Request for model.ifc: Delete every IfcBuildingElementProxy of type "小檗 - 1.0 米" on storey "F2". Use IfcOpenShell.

First a look at what the model holds.

```python
import ifcopenshell
import ifcopenshell.util.element

model = ifcopenshell.open("model.ifc")
print(model.schema)
storey = next(s for s in model.by_type("IfcBuildingStorey") if s.Name == "F2")
proxies = [e for e in ifcopenshell.util.element.get_decomposition(storey) if e.is_a("IfcBuildingElementProxy")]
seen = {}
for e in proxies:
    element_type = ifcopenshell.util.element.get_type(e)
    name = element_type.Name if element_type not in (None, e) else None
    seen[name] = seen.get(name, 0) + 1
for name, count in sorted(seen.items(), key=str):
    print(count, "x", name)
```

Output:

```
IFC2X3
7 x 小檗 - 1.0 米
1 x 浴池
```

```python
import ifcopenshell
import ifcopenshell.api.root
import ifcopenshell.util.element

model = ifcopenshell.open("model.ifc")

storey = next(s for s in model.by_type("IfcBuildingStorey") if s.Name == "F2")
proxies = [e for e in ifcopenshell.util.element.get_decomposition(storey) if e.is_a("IfcBuildingElementProxy")]
targets = [e for e in proxies if (t := ifcopenshell.util.element.get_type(e)) not in (None, e) and t.Name == "小檗 - 1.0 米"]

for e in targets:
    ifcopenshell.api.root.remove_product(model, product=e)
print(len(targets), "removed")

model.write("model-out.ifc")
```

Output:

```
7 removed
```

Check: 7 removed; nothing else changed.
